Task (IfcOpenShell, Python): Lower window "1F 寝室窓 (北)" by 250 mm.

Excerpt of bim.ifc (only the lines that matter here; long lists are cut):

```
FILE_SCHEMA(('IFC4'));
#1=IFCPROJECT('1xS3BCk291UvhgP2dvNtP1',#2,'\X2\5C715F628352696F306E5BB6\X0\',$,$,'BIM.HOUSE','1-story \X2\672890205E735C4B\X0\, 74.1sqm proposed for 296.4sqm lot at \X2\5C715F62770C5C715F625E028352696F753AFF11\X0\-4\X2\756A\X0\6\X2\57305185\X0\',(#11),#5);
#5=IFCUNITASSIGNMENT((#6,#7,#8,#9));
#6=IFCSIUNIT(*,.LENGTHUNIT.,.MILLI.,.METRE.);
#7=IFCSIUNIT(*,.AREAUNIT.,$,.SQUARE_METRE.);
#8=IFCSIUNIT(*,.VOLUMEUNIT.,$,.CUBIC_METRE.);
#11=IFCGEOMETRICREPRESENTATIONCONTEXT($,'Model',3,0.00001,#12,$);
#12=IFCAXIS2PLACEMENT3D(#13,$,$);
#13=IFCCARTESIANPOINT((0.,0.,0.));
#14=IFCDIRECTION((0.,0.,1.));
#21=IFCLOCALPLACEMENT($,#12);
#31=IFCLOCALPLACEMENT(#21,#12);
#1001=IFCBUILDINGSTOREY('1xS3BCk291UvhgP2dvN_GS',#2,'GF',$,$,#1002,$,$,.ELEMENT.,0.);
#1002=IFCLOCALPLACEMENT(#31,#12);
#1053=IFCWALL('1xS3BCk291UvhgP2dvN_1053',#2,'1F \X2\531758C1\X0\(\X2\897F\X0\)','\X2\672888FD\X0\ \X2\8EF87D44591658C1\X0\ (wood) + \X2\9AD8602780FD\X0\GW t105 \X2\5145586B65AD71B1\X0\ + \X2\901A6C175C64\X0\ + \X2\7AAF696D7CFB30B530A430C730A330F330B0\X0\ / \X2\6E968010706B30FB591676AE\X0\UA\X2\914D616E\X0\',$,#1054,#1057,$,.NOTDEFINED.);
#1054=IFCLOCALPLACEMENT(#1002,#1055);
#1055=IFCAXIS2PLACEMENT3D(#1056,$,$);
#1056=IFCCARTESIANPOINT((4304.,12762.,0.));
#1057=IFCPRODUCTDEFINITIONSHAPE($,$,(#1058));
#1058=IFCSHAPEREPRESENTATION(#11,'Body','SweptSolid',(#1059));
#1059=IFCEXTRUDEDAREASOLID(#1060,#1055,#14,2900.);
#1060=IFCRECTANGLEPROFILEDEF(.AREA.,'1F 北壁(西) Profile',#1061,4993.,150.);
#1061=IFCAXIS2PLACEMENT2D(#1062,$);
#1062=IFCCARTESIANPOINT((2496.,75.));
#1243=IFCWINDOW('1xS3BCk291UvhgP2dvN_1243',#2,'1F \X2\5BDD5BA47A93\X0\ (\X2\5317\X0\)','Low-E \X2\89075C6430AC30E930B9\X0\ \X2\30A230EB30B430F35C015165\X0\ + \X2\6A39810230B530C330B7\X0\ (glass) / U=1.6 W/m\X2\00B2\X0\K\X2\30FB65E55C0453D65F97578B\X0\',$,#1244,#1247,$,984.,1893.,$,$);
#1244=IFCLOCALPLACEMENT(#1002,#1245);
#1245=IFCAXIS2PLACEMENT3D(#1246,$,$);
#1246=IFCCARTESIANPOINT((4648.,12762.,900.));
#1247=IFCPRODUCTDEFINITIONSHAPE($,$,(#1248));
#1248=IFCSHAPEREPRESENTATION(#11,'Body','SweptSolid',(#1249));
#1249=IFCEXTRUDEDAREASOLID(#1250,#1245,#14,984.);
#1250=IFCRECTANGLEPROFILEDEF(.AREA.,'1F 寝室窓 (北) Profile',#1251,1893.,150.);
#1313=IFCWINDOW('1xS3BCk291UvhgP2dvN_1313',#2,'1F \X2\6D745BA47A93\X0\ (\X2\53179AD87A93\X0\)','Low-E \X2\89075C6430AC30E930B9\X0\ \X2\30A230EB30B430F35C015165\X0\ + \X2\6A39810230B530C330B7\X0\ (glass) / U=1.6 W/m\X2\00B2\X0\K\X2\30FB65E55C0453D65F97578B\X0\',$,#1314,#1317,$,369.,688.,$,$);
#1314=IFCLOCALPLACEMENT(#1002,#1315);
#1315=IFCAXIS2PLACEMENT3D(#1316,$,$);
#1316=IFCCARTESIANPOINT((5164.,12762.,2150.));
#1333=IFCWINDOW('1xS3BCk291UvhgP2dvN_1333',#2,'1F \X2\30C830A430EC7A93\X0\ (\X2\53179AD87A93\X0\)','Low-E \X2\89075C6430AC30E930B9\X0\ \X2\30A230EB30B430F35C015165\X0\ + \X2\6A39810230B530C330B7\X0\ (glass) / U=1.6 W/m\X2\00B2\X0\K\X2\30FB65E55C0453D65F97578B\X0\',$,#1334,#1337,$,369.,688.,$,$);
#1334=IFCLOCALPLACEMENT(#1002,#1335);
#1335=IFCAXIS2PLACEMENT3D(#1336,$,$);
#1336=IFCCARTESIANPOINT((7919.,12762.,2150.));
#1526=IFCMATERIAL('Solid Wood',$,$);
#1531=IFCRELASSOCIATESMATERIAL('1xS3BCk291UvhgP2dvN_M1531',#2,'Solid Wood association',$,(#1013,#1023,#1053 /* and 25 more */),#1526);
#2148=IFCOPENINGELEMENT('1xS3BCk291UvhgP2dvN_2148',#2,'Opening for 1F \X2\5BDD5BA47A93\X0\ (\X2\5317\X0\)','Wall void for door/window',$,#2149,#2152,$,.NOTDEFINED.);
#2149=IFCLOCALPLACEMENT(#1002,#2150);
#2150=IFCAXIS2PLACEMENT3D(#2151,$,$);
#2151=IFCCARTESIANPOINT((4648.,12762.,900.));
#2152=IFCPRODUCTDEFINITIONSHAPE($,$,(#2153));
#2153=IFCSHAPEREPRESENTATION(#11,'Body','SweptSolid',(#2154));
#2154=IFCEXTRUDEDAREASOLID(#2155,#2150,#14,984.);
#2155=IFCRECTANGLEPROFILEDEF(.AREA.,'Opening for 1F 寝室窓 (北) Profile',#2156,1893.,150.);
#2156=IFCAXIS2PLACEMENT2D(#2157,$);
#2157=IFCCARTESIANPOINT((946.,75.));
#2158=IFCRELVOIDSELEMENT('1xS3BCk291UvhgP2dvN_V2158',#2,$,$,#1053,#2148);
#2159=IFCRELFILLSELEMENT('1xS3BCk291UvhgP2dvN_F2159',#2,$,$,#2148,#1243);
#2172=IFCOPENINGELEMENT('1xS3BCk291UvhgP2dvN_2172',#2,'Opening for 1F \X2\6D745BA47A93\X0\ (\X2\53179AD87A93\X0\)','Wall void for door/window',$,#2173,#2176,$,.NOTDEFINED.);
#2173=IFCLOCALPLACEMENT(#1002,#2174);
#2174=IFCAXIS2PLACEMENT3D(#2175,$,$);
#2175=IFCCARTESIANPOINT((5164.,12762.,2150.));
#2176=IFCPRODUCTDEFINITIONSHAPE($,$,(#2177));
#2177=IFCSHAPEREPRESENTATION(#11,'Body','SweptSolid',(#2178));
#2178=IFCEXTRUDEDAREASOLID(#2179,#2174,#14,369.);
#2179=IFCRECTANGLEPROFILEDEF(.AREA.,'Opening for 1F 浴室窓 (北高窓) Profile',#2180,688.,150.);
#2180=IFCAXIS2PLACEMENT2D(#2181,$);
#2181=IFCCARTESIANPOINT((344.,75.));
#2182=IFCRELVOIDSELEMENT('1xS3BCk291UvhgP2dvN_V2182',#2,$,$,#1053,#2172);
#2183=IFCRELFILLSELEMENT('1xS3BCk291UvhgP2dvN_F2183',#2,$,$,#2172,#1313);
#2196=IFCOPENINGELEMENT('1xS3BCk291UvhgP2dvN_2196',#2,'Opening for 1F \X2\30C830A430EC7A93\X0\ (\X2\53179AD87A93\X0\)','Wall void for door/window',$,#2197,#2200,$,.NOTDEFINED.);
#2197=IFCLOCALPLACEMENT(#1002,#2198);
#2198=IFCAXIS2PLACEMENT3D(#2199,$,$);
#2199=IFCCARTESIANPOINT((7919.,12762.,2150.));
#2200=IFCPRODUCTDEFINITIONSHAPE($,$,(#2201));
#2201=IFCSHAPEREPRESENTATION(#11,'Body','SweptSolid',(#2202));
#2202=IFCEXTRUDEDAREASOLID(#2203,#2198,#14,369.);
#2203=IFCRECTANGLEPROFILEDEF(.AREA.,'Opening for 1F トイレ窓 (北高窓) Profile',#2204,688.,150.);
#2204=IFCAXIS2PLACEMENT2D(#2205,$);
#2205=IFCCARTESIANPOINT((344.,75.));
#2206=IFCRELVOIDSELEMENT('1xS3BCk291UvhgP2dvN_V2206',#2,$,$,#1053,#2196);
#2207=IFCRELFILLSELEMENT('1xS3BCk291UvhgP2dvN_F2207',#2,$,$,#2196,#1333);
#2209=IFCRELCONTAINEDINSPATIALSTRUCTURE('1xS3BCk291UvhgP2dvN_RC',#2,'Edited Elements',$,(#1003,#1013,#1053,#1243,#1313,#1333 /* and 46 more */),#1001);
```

```python
import numpy as np
import ifcopenshell
import ifcopenshell.api.geometry
import ifcopenshell.util.placement
import ifcopenshell.util.unit

model = ifcopenshell.open("bim.ifc")
unit_scale = ifcopenshell.util.unit.calculate_unit_scale(model)

window = model.by_guid("1xS3BCk291UvhgP2dvN_1243")
opening = window.FillsVoids[0].RelatingOpeningElement
dz = -0.25 / unit_scale

shift = np.array([0.0, 0.0, dz])
# The window is not placed relative to its opening, so move both.
for product in (opening, window):
    matrix = ifcopenshell.util.placement.get_local_placement(product.ObjectPlacement)
    matrix[:3, 3] += shift
    ifcopenshell.api.geometry.edit_object_placement(model, product=product, matrix=matrix, is_si=False)

print(f"moved by {dz * unit_scale:+.3f} m")

model.write("bim-out.ifc")
```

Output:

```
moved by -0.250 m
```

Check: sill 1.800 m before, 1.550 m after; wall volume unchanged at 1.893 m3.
